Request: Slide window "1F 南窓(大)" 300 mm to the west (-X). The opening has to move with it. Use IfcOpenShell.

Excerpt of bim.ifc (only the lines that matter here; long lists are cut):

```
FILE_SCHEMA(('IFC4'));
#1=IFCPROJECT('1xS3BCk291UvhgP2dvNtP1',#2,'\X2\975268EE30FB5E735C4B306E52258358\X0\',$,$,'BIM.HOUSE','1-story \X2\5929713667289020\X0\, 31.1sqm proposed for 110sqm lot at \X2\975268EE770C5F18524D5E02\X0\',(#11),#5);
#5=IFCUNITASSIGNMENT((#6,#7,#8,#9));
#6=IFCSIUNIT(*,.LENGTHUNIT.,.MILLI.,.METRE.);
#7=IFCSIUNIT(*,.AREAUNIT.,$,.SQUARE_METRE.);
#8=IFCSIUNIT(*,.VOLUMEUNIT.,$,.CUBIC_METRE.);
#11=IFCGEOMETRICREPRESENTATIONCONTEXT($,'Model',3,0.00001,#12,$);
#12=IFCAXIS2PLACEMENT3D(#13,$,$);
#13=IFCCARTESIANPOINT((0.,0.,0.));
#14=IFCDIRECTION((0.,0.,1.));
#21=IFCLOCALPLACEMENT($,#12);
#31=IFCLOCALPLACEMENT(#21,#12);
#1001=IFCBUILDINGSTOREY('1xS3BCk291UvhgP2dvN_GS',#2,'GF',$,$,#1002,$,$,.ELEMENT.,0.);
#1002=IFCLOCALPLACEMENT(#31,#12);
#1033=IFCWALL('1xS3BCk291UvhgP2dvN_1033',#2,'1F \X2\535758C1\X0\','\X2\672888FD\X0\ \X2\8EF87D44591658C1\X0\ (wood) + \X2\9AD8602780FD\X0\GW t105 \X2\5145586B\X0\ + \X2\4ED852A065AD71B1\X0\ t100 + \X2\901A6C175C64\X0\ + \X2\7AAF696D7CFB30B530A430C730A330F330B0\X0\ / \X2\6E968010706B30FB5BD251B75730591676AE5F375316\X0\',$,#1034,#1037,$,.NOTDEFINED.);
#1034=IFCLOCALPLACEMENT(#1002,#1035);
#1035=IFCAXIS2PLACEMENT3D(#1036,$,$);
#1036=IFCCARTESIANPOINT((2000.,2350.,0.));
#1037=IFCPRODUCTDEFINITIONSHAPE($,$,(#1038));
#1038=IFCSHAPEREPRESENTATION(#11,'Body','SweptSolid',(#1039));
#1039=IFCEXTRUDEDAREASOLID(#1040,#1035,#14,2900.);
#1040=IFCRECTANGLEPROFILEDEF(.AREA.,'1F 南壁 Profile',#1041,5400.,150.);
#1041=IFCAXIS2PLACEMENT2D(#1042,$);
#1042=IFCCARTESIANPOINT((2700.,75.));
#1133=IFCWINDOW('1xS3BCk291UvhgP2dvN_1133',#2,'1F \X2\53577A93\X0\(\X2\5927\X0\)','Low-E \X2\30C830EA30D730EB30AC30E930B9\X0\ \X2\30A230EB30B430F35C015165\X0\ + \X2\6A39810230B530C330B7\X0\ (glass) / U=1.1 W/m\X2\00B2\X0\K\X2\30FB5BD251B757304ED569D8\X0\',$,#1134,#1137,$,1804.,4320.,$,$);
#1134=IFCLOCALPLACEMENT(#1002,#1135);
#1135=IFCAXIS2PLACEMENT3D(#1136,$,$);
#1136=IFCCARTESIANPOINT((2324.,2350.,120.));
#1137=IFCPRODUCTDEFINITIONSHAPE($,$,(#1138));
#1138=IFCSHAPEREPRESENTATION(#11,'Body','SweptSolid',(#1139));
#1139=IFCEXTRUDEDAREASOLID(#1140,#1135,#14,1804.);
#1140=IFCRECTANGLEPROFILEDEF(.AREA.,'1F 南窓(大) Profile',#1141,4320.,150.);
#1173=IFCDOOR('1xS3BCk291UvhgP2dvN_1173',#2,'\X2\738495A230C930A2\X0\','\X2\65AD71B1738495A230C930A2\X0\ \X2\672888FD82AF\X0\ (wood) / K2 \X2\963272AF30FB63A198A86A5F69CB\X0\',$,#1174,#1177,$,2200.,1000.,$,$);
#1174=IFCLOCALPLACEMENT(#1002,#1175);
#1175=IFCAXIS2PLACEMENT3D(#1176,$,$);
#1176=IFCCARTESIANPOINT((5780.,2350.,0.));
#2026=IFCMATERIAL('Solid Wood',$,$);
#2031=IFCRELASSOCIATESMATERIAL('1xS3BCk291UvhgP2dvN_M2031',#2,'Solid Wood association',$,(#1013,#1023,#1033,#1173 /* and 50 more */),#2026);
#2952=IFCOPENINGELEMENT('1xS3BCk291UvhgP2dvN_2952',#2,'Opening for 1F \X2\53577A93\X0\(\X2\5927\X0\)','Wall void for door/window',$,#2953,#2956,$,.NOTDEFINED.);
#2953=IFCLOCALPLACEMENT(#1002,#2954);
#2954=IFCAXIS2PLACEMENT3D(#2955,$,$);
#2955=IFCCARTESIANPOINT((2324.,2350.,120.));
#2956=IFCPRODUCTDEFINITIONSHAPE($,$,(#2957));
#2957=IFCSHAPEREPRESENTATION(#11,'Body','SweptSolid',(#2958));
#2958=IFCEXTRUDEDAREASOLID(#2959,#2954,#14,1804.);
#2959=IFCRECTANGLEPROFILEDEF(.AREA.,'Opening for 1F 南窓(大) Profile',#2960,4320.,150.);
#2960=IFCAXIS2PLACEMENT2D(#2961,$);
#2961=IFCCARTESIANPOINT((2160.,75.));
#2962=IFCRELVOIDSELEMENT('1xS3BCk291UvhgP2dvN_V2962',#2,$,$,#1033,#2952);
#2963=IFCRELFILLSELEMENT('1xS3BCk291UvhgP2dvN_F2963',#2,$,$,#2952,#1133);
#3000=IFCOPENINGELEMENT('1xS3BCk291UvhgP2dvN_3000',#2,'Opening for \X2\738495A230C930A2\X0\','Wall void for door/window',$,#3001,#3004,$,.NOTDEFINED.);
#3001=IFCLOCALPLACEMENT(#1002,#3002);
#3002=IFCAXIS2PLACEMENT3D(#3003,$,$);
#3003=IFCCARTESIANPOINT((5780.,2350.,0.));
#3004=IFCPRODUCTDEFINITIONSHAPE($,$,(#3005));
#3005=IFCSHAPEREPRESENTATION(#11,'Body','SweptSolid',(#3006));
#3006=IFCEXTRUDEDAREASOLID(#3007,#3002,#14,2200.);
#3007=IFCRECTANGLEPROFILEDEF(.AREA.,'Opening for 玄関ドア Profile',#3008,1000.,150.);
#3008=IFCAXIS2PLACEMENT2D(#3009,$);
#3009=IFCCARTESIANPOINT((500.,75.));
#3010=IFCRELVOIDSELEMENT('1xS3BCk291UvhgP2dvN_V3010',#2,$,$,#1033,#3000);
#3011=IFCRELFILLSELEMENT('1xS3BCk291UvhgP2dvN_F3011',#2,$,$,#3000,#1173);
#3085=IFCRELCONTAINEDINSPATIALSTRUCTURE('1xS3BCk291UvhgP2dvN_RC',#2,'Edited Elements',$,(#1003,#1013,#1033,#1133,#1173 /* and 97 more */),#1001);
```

```python
import ifcopenshell
import ifcopenshell.api.geometry
import ifcopenshell.util.placement

model = ifcopenshell.open("bim.ifc")

window = model.by_guid("1xS3BCk291UvhgP2dvN_1133")
opening = window.FillsVoids[0].RelatingOpeningElement
wall = opening.VoidsElements[0].RelatingBuildingElement

wall_matrix = ifcopenshell.util.placement.get_local_placement(wall.ObjectPlacement)
shift = wall_matrix[:3, 0] * -300.0
before = ifcopenshell.util.placement.get_local_placement(window.ObjectPlacement)[:3, 3].copy()

# The window is not placed relative to its opening, so move both.
for product in (opening, window):
    matrix = ifcopenshell.util.placement.get_local_placement(product.ObjectPlacement)
    matrix[:3, 3] += shift
    ifcopenshell.api.geometry.edit_object_placement(model, product=product, matrix=matrix, is_si=False)

after = ifcopenshell.util.placement.get_local_placement(window.ObjectPlacement)[:3, 3]
print("window moved by", (after - before).round(3) + 0.0)

model.write("bim_rev.ifc")
```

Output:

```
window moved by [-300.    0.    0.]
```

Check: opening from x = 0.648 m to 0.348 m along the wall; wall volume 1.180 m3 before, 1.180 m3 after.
